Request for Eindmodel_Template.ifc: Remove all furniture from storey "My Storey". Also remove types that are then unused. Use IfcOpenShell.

First a look at what the model holds.

```python
import ifcopenshell
import ifcopenshell.util.element

model = ifcopenshell.open("Eindmodel_Template.ifc")
print(model.schema)
storey = next(s for s in model.by_type("IfcBuildingStorey") if s.Name == "My Storey")
furniture = [e for e in ifcopenshell.util.element.get_decomposition(storey) if e.is_a("IfcFurnishingElement")]
seen = {}
for e in furniture:
    element_type = ifcopenshell.util.element.get_type(e)
    name = element_type.Name if element_type not in (None, e) else None
    seen[name] = seen.get(name, 0) + 1
for name, count in sorted(seen.items(), key=str):
    print(count, "x", name)
```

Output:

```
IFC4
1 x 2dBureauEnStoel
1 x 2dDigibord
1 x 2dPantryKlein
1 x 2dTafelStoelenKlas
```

```python
import ifcopenshell
import ifcopenshell.api.root
import ifcopenshell.util.element

model = ifcopenshell.open("Eindmodel_Template.ifc")

storey = next(s for s in model.by_type("IfcBuildingStorey") if s.Name == "My Storey")
furniture = [e for e in ifcopenshell.util.element.get_decomposition(storey) if e.is_a("IfcFurnishingElement")]
types = {ifcopenshell.util.element.get_type(e) for e in furniture} - {None, *furniture}

for e in furniture:
    ifcopenshell.api.root.remove_product(model, product=e)
print(len(furniture), "removed")

unused = [t for t in types if not ifcopenshell.util.element.get_types(t)]
for t in unused:
    ifcopenshell.api.root.remove_product(model, product=t)
print(len(unused), "unused types removed")

model.write("Eindmodel_Template_rev.ifc")
```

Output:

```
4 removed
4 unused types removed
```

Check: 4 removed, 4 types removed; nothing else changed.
